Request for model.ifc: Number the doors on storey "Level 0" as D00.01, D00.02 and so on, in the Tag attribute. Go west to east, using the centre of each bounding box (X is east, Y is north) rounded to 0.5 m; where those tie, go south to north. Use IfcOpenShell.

First a look at what the model holds.

```python
import ifcopenshell
import ifcopenshell.util.element
import ifcopenshell.util.placement

model = ifcopenshell.open("model.ifc")
print(model.schema)
storey = next(s for s in model.by_type("IfcBuildingStorey") if s.Name == "Level 0")
doors = [e for e in ifcopenshell.util.element.get_decomposition(storey) if e.is_a("IfcDoor")]
for e in sorted(doors, key=lambda e: e.id()):
    origin = ifcopenshell.util.placement.get_local_placement(e.ObjectPlacement)[:3, 3]
    print(e.id(), e.Tag, e.Name, origin.round(2) + 0.0, sep=" | ")
```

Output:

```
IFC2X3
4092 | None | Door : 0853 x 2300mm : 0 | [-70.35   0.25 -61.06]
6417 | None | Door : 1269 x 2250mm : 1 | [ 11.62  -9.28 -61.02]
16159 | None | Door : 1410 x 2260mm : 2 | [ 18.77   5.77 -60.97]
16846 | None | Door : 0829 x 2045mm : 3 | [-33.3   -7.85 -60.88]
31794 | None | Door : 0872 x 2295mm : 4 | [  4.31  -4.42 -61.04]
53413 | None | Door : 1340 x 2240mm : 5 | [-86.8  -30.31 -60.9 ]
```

```python
import ifcopenshell
import ifcopenshell.geom
import ifcopenshell.util.element
import ifcopenshell.util.shape

model = ifcopenshell.open("model.ifc")
settings = ifcopenshell.geom.settings()
settings.set("use-world-coords", True)


def centre(element):
    shape = ifcopenshell.geom.create_shape(settings, element)
    return ifcopenshell.util.shape.get_bbox_centroid(shape.geometry)


storey = next(s for s in model.by_type("IfcBuildingStorey") if s.Name == "Level 0")
doors = [e for e in ifcopenshell.util.element.get_decomposition(storey) if e.is_a("IfcDoor")]

# Insertion points can sit at a corner or the storey origin, so sort by the geometry (in metres).
centres = {e: centre(e) for e in doors}
doors.sort(key=lambda e: (round(centres[e][0] / 0.5), centres[e][1]))

for i, e in enumerate(doors, start=1):
    number = f"D00.{i:02d}"
    e.Tag = number
    print(e.id(), number)

model.write("model_rev.ifc")
```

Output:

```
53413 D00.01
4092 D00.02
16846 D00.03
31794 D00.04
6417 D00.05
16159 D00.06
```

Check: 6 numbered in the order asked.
